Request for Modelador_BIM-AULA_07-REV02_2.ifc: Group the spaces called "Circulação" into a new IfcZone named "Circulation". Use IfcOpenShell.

First a look at what the model holds.

```python
import ifcopenshell

model = ifcopenshell.open("Modelador_BIM-AULA_07-REV02_2.ifc")
print(model.schema)
seen = {}
for space in model.by_type("IfcSpace"):
    seen[space.LongName] = seen.get(space.LongName, 0) + 1
for name, count in sorted(seen.items(), key=str):
    print(count, "x", name)
print("zones:", [z.Name for z in model.by_type("IfcZone")][:20])
```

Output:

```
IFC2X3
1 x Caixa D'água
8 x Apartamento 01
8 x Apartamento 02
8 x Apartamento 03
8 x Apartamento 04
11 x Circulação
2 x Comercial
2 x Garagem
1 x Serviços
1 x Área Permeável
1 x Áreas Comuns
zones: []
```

```python
import ifcopenshell
import ifcopenshell.api.group
import ifcopenshell.api.root

model = ifcopenshell.open("Modelador_BIM-AULA_07-REV02_2.ifc")

names = {"Circulação"}
spaces = [s for s in model.by_type("IfcSpace") if s.LongName in names]

zone = ifcopenshell.api.root.create_entity(model, ifc_class="IfcZone", name="Circulation")
ifcopenshell.api.group.assign_group(model, products=spaces, group=zone)
print(len(spaces), "spaces in", zone.Name)

model.write("Modelador_BIM-AULA_07-REV02_2_edited.ifc")
```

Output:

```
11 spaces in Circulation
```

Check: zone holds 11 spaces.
